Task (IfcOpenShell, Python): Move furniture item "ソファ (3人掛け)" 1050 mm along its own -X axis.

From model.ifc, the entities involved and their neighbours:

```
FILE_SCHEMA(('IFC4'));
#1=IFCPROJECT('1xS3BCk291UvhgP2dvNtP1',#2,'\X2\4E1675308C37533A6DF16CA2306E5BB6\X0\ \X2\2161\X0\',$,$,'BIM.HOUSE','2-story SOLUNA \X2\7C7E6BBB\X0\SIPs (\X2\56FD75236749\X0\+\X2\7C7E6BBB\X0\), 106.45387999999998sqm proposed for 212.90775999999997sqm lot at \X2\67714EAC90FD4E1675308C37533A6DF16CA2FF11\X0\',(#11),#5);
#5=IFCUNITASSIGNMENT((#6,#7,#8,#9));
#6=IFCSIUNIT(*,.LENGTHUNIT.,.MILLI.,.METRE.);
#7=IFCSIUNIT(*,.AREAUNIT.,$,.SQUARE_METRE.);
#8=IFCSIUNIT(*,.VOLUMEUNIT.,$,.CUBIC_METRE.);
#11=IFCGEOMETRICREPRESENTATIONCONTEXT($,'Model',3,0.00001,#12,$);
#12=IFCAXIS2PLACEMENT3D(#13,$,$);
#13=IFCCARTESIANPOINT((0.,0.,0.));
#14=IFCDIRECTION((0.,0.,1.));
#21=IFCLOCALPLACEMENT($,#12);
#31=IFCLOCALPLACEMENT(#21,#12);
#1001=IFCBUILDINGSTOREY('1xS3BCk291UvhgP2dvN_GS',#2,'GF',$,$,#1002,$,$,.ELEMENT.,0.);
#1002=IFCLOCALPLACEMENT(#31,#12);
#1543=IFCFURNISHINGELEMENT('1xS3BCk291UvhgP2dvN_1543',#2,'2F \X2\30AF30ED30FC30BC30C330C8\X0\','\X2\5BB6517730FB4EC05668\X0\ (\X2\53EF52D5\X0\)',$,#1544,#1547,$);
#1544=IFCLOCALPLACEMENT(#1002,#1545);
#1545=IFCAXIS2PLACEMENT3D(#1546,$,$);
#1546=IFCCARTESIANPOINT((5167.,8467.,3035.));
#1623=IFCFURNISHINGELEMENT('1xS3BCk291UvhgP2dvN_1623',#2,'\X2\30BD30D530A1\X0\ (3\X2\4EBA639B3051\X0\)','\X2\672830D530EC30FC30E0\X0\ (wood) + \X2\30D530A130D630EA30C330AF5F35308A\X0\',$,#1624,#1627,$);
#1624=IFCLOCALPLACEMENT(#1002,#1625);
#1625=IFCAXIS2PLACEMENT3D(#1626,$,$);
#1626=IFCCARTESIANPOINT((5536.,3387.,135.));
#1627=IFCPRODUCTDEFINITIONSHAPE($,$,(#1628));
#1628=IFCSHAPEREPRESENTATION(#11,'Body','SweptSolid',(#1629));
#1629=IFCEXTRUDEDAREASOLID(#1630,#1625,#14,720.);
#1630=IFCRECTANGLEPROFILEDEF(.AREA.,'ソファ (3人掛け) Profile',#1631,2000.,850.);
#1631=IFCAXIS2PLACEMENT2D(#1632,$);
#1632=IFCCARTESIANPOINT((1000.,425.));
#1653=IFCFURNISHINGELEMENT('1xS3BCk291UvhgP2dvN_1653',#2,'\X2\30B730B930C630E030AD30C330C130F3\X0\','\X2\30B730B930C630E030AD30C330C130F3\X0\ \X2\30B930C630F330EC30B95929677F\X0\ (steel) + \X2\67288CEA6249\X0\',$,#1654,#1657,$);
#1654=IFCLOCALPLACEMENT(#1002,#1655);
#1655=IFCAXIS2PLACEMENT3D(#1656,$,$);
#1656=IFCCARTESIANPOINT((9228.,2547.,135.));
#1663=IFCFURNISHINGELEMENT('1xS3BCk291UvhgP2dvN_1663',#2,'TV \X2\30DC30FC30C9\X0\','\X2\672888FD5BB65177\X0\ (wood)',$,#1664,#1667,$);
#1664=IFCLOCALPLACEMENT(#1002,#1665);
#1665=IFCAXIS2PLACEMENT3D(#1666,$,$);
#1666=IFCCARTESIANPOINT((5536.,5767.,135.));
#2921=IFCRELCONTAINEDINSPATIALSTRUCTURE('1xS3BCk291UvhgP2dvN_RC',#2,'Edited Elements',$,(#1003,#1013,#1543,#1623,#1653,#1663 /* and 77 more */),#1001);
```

```python
import ifcopenshell
import ifcopenshell.api.geometry
import ifcopenshell.util.placement

model = ifcopenshell.open("model.ifc")

item = model.by_guid("1xS3BCk291UvhgP2dvN_1623")
matrix = ifcopenshell.util.placement.get_local_placement(item.ObjectPlacement)
matrix[:3, 3] -= matrix[:3, 0] * 1050.0
ifcopenshell.api.geometry.edit_object_placement(model, product=item, matrix=matrix, is_si=False)

print(ifcopenshell.util.placement.get_local_placement(item.ObjectPlacement).round(3) + 0.0)

model.write("model_updated.ifc")
```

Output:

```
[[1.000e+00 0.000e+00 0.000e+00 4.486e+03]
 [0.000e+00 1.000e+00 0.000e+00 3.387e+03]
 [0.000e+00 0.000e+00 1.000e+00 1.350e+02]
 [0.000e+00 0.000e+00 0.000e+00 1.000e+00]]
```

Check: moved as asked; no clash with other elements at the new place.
